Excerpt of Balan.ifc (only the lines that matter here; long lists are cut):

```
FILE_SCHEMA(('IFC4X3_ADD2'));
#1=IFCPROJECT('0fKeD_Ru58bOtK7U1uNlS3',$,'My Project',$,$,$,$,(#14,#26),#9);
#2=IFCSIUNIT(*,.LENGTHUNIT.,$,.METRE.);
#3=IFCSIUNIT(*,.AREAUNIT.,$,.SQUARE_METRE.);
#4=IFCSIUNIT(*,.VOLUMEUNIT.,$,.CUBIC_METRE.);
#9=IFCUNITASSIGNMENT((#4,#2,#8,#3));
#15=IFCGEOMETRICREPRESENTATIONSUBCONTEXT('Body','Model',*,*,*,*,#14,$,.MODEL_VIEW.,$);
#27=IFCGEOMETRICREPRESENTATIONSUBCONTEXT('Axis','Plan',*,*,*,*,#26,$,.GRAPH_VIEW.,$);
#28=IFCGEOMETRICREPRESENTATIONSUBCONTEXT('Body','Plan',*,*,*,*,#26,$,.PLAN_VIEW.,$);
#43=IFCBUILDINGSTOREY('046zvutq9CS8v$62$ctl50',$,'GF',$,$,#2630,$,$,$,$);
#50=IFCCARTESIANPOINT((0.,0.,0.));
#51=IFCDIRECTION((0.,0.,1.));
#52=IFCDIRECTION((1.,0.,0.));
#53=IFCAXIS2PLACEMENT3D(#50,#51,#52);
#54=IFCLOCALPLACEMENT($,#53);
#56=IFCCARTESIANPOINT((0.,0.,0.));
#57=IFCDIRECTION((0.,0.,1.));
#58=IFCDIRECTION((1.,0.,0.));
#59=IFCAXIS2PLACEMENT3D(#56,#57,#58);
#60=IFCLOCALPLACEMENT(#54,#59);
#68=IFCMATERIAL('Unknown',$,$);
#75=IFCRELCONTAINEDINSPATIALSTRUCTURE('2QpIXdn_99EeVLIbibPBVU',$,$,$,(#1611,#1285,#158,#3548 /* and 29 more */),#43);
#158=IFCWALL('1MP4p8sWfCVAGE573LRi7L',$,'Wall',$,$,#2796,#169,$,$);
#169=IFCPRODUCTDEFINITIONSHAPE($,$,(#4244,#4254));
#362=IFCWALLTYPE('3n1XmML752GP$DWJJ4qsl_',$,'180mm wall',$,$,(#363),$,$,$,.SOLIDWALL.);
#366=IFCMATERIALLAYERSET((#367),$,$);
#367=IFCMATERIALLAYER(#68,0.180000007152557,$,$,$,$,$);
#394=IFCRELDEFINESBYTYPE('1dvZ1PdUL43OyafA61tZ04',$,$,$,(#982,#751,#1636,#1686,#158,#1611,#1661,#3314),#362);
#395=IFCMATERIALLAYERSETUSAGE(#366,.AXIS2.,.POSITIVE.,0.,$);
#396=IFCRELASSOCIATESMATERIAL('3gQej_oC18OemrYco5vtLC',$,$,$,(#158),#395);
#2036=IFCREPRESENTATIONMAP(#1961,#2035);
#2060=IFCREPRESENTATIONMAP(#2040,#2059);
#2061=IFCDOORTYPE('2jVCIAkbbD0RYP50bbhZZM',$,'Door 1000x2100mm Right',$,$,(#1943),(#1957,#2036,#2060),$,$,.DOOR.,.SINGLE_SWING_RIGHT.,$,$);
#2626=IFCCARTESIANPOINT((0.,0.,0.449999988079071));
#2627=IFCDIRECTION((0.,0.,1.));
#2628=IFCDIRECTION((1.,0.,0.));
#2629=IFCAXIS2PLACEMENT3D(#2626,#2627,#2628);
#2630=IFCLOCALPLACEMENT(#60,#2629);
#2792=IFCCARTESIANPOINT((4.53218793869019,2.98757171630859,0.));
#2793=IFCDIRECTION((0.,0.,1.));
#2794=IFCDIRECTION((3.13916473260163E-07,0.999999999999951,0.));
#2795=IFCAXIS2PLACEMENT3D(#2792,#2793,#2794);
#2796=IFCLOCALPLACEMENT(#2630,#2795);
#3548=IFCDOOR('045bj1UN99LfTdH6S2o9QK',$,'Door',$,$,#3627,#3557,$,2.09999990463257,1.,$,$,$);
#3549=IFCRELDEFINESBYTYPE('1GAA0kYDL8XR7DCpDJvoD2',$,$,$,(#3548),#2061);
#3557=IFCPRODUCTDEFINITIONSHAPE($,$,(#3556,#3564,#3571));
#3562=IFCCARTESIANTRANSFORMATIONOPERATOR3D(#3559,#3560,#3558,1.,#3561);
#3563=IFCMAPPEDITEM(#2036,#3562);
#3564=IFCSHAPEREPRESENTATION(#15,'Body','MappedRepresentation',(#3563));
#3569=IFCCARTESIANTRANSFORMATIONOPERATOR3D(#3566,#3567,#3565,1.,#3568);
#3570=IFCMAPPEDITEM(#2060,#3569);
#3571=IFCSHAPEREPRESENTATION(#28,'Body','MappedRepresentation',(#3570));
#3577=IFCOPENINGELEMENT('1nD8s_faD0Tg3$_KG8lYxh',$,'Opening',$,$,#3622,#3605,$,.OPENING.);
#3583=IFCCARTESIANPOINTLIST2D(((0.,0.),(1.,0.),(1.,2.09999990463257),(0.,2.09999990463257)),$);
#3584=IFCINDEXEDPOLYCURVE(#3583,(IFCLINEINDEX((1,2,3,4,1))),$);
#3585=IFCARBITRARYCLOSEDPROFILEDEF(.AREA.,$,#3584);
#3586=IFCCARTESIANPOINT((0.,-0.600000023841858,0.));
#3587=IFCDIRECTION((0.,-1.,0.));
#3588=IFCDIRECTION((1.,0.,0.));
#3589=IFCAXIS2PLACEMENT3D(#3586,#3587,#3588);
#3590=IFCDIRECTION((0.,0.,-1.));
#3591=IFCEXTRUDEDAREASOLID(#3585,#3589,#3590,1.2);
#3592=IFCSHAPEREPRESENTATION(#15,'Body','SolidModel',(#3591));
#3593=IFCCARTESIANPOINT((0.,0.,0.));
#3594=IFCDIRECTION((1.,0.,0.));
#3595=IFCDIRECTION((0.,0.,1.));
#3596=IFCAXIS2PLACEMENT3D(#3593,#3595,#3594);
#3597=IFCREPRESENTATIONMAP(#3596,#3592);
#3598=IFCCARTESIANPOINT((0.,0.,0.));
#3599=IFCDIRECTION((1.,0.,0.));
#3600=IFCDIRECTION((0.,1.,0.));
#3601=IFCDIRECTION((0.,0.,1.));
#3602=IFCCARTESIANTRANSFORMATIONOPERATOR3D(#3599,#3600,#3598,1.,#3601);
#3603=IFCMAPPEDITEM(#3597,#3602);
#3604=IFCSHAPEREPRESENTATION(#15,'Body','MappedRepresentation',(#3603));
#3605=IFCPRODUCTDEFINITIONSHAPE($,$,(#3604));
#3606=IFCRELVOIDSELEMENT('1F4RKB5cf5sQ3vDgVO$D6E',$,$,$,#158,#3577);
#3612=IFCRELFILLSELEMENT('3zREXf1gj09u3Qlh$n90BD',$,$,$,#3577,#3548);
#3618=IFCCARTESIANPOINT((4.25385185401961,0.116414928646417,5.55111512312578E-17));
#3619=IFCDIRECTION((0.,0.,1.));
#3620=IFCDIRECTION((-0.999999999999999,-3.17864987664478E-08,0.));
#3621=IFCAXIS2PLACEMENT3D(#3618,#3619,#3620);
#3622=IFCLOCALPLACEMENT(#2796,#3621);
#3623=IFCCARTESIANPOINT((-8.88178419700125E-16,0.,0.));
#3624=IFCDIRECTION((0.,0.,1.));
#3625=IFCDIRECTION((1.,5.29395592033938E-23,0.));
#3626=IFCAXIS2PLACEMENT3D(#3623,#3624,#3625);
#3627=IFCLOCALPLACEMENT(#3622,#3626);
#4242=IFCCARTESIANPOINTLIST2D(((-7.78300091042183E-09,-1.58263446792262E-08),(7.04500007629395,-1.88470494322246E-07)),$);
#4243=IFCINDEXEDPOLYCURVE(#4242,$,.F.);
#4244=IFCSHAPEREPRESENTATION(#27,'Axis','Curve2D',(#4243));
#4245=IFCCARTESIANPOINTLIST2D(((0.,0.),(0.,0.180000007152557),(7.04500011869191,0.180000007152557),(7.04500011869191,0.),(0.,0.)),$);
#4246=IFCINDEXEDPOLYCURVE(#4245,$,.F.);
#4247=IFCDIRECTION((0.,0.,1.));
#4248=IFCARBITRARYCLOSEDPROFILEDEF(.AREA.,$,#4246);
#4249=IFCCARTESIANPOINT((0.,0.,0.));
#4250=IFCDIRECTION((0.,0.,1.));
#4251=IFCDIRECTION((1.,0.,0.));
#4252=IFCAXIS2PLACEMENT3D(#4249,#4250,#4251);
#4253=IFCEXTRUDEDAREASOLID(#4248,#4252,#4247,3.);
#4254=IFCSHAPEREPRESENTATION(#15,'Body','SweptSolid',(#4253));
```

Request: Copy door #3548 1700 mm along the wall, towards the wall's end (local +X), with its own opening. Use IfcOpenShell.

```python
import ifcopenshell
import ifcopenshell.api.feature
import ifcopenshell.api.geometry
import ifcopenshell.api.root
import ifcopenshell.geom
import ifcopenshell.util.element
import ifcopenshell.util.placement
import ifcopenshell.util.shape

model = ifcopenshell.open("Balan.ifc")
settings = ifcopenshell.geom.settings()


def volume(element):
    """Net volume in cubic metres, openings subtracted."""
    shape = ifcopenshell.geom.create_shape(settings, element)
    return ifcopenshell.util.shape.get_volume(shape.geometry)


door = model.by_guid("045bj1UN99LfTdH6S2o9QK")
opening = door.FillsVoids[0].RelatingOpeningElement
wall = opening.VoidsElements[0].RelatingBuildingElement
before = volume(wall)
shift = ifcopenshell.util.placement.get_local_placement(wall.ObjectPlacement)[:3, 0] * 1.7

# copy_class copies the void relationship, type, container and properties, but no geometry.
new_opening = ifcopenshell.api.root.copy_class(model, product=opening)
new_opening.Representation = ifcopenshell.util.element.copy_deep(
    model, opening.Representation, exclude=["IfcGeometricRepresentationContext", "IfcRepresentationMap"]
)
new_door = ifcopenshell.api.root.copy_class(model, product=door)
new_door.Representation = ifcopenshell.util.element.copy_deep(
    model, door.Representation, exclude=["IfcGeometricRepresentationContext", "IfcRepresentationMap"]
)
ifcopenshell.api.feature.add_filling(model, opening=new_opening, element=new_door)

for old, new in ((opening, new_opening), (door, new_door)):
    matrix = ifcopenshell.util.placement.get_local_placement(old.ObjectPlacement)
    matrix[:3, 3] += shift
    ifcopenshell.api.geometry.edit_object_placement(model, product=new, matrix=matrix, is_si=False)

after = volume(wall)

print(f"wall volume {before:.3f} -> {after:.3f} m3")

model.write("Balan_updated.ifc")
```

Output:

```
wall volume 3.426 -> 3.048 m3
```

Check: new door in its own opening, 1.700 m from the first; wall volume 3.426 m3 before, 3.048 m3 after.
